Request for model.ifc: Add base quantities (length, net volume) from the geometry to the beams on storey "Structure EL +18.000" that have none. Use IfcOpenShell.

First a look at what the model holds.

```python
import ifcopenshell
import ifcopenshell.util.element
import ifcopenshell.util.unit

model = ifcopenshell.open("model.ifc")
print(model.schema)
for unit_type in ("LENGTHUNIT", "AREAUNIT", "VOLUMEUNIT"):
    print(unit_type, ifcopenshell.util.unit.calculate_unit_scale(model, unit_type))
storey = next(s for s in model.by_type("IfcBuildingStorey") if s.Name == "Structure EL +18.000")
beams = [e for e in ifcopenshell.util.element.get_decomposition(storey) if e.is_a("IfcBeam")]
for e in sorted(beams, key=lambda e: e.id()):
    print(e.id(), e.is_a(), e.Name, list(ifcopenshell.util.element.get_psets(e, qtos_only=True)), sep=" | ")
```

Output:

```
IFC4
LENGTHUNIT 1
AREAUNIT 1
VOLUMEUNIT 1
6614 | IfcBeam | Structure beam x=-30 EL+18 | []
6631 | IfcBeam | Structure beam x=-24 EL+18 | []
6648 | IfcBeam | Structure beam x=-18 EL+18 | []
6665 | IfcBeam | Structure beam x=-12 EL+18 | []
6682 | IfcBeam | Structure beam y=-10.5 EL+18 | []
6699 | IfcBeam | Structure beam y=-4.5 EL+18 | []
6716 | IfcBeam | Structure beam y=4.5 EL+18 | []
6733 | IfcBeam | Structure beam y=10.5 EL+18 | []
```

```python
import ifcopenshell
import ifcopenshell.api.pset
import ifcopenshell.geom
import ifcopenshell.util.element
import ifcopenshell.util.shape
import ifcopenshell.util.unit

model = ifcopenshell.open("model.ifc")
unit_scale = ifcopenshell.util.unit.calculate_unit_scale(model)
volume_scale = ifcopenshell.util.unit.calculate_unit_scale(model, "VOLUMEUNIT")
settings = ifcopenshell.geom.settings()

storey = next(s for s in model.by_type("IfcBuildingStorey") if s.Name == "Structure EL +18.000")
beams = [e for e in ifcopenshell.util.element.get_decomposition(storey) if e.is_a("IfcBeam")]

for e in sorted(beams, key=lambda e: e.id()):
    if ifcopenshell.util.element.get_psets(e, qtos_only=True, should_inherit=False):
        continue
    # Geometry comes back in metres, in the element's own axes.
    shape = ifcopenshell.geom.create_shape(settings, e)
    values = {
        "Length": ifcopenshell.util.shape.get_max_xyz(shape.geometry) / unit_scale,
        "NetVolume": ifcopenshell.util.shape.get_volume(shape.geometry) / volume_scale,
    }
    qto = ifcopenshell.api.pset.add_qto(model, product=e, name="Qto_BeamBaseQuantities")
    ifcopenshell.api.pset.edit_qto(model, qto=qto, properties=values)
    print(e.id(), {k: round(v, 3) for k, v in values.items()})

model.write("model-out.ifc")
```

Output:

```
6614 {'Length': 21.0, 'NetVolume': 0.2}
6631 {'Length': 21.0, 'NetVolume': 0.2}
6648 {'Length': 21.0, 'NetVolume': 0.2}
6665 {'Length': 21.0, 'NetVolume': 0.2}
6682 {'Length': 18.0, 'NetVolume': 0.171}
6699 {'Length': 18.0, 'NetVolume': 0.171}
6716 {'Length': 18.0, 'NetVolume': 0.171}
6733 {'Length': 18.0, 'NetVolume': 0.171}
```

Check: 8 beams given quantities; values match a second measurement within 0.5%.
